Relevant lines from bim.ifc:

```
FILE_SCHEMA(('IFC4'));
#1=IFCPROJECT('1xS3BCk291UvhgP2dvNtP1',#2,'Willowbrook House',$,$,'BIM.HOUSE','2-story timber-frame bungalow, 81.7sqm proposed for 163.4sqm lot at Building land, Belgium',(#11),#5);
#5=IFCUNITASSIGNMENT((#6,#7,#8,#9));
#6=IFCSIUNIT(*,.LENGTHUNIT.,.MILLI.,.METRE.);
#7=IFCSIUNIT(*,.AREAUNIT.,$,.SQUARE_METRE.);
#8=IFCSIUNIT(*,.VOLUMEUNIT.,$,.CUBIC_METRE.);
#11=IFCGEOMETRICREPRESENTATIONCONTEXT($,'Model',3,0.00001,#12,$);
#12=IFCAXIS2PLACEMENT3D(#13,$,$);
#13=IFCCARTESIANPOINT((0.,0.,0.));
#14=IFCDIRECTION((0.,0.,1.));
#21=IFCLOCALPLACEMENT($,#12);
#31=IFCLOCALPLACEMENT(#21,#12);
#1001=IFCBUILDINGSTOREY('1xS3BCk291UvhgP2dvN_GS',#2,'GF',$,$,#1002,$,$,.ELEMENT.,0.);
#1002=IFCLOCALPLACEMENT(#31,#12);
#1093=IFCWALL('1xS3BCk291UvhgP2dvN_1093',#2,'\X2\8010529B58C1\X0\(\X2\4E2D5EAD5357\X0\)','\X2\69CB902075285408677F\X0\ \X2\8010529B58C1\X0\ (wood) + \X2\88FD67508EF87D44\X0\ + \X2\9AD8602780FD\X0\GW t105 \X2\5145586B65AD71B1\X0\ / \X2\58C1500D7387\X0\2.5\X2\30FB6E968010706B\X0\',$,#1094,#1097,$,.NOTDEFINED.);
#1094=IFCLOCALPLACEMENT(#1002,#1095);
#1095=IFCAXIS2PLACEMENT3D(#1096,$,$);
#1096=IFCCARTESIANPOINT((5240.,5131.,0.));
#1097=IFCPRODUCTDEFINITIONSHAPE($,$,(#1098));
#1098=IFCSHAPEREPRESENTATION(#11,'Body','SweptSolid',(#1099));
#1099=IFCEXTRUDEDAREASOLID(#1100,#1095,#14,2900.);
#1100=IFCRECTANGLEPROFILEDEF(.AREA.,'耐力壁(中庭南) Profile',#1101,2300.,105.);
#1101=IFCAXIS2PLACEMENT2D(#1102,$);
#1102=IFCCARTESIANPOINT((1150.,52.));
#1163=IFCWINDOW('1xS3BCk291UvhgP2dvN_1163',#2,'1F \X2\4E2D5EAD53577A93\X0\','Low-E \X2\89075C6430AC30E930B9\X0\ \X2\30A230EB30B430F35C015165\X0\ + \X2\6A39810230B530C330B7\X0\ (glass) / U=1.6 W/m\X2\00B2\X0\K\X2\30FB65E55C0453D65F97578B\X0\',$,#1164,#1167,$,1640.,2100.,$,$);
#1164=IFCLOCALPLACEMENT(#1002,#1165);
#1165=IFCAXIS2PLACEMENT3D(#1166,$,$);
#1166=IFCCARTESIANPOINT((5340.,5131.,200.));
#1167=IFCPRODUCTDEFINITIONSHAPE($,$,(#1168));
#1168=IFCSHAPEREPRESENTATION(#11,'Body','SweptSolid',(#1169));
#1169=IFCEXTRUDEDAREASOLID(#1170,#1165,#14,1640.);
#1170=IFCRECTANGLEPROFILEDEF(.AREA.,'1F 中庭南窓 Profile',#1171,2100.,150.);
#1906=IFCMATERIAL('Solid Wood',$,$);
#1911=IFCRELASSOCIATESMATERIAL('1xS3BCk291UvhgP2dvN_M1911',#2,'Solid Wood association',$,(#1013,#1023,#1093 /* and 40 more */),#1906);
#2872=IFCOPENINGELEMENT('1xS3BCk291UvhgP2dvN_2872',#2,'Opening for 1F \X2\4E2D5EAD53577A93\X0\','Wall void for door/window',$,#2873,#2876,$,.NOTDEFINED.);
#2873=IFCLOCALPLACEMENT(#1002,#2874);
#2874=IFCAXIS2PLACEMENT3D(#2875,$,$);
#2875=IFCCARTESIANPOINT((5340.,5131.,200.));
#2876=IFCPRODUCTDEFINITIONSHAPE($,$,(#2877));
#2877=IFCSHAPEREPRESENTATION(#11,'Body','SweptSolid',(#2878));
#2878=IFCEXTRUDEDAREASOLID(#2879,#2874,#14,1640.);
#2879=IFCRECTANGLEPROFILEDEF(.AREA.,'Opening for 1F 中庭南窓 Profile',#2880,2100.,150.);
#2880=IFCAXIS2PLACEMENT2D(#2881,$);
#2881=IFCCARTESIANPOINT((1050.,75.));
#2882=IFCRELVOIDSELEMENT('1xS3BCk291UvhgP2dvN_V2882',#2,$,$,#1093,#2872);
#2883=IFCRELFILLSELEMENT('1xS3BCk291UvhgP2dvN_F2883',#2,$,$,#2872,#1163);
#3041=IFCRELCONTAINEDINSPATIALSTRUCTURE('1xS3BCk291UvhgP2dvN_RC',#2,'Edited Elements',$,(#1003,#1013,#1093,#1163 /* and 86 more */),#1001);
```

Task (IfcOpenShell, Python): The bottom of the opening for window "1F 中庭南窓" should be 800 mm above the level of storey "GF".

```python
import numpy as np
import ifcopenshell
import ifcopenshell.api.geometry
import ifcopenshell.geom
import ifcopenshell.util.element
import ifcopenshell.util.placement
import ifcopenshell.util.shape
import ifcopenshell.util.unit

model = ifcopenshell.open("bim.ifc")
unit_scale = ifcopenshell.util.unit.calculate_unit_scale(model)

window = model.by_id(1163)
opening = window.FillsVoids[0].RelatingOpeningElement
storey = ifcopenshell.util.element.get_container(window, ifc_class="IfcBuildingStorey")
level = ifcopenshell.util.placement.get_local_placement(storey.ObjectPlacement)[2, 3]

# The opening's origin need not be at the sill, so measure its lowest point.
shape = ifcopenshell.geom.create_shape(ifcopenshell.geom.settings(), opening)
bottom = ifcopenshell.util.shape.get_shape_bottom_elevation(shape, shape.geometry) / unit_scale
dz = level + 800.0 - bottom

shift = np.array([0.0, 0.0, dz])
# The window is not placed relative to its opening, so move both.
for product in (opening, window):
    matrix = ifcopenshell.util.placement.get_local_placement(product.ObjectPlacement)
    matrix[:3, 3] += shift
    ifcopenshell.api.geometry.edit_object_placement(model, product=product, matrix=matrix, is_si=False)

print(f"moved by {dz * unit_scale:+.3f} m")

model.write("bim-out.ifc")
```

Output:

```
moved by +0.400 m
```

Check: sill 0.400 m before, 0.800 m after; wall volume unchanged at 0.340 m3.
